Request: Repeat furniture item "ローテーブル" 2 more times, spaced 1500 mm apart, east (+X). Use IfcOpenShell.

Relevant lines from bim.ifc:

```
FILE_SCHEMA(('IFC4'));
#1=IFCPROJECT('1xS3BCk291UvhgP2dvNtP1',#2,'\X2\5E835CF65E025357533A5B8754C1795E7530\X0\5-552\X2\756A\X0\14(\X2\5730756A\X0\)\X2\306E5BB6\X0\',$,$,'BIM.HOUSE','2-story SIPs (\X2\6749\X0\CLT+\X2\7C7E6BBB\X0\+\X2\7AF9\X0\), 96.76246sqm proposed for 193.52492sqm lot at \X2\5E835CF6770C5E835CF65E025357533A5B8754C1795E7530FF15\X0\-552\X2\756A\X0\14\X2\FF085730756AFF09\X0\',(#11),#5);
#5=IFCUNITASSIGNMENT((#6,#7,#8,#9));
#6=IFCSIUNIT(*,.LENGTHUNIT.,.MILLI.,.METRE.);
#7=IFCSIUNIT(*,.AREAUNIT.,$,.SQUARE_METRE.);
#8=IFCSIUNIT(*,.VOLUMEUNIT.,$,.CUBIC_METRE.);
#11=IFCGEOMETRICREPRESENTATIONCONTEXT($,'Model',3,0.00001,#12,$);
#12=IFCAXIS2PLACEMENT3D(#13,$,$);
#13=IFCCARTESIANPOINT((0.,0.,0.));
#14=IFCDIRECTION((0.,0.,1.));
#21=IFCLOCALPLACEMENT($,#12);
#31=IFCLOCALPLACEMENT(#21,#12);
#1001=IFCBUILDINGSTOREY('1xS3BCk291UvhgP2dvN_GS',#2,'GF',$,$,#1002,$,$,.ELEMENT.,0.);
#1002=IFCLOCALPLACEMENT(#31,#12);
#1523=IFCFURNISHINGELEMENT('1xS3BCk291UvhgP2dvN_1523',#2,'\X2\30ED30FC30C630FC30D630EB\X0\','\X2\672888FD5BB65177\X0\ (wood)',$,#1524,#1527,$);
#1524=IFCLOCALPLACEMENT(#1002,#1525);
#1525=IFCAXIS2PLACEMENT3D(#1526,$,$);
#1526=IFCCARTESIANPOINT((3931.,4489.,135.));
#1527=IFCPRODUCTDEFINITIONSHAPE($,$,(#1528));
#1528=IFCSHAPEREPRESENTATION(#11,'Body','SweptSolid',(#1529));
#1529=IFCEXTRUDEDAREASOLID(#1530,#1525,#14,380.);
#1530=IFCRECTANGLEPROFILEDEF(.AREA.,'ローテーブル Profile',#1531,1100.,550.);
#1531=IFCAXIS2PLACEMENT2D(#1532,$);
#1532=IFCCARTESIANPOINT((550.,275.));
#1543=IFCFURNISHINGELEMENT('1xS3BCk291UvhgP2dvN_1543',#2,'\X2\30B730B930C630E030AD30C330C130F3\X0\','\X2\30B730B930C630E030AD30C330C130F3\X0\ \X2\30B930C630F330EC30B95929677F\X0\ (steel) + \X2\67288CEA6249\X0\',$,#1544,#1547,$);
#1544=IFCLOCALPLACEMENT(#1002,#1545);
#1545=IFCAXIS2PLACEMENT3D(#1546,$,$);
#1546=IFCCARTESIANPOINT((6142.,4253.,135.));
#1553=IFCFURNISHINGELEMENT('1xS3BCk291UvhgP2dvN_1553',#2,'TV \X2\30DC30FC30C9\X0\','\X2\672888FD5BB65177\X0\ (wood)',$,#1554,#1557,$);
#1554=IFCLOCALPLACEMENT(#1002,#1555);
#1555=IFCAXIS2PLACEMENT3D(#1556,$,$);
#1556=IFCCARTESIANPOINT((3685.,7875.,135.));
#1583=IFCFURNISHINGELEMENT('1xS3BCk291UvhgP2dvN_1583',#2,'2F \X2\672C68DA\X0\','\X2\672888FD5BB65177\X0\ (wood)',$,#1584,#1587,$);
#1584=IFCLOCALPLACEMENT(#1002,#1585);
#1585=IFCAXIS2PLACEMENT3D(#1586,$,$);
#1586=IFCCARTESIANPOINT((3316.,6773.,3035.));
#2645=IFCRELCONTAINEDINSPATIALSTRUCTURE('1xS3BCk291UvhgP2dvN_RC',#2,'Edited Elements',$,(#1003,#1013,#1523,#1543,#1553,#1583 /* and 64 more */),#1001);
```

```python
import numpy as np
import ifcopenshell
import ifcopenshell.api.geometry
import ifcopenshell.api.root
import ifcopenshell.util.element
import ifcopenshell.util.placement
import ifcopenshell.util.unit

model = ifcopenshell.open("bim.ifc")
unit_scale = ifcopenshell.util.unit.calculate_unit_scale(model)


def reuse_history(source, copy):
    """copy_class also copies each property set's owner history, people and application; keep the originals."""
    for rel in copy.IsDefinedBy:
        if rel.is_a("IfcRelDefinesByProperties") and (history := rel.RelatingPropertyDefinition.OwnerHistory):
            rel.RelatingPropertyDefinition.OwnerHistory = source.OwnerHistory
            ifcopenshell.util.element.remove_deep2(model, history)


source = model.by_guid("1xS3BCk291UvhgP2dvN_1523")
base = ifcopenshell.util.placement.get_local_placement(source.ObjectPlacement)
step = np.array([1.0, 0.0, 0.0]) * 1.5 / unit_scale

for i in range(1, 3):
    copy = ifcopenshell.api.root.copy_class(model, product=source)
    copy.Representation = ifcopenshell.util.element.copy_deep(
        model, source.Representation, exclude=["IfcGeometricRepresentationContext", "IfcRepresentationMap"]
    )
    reuse_history(source, copy)
    matrix = base.copy()
    matrix[:3, 3] += i * step
    print("added at", matrix[:3, 3].round(3) + 0.0)
    ifcopenshell.api.geometry.edit_object_placement(model, product=copy, matrix=matrix, is_si=False)

model.write("bim_updated.ifc")
```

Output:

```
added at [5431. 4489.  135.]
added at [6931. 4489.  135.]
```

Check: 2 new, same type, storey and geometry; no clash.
